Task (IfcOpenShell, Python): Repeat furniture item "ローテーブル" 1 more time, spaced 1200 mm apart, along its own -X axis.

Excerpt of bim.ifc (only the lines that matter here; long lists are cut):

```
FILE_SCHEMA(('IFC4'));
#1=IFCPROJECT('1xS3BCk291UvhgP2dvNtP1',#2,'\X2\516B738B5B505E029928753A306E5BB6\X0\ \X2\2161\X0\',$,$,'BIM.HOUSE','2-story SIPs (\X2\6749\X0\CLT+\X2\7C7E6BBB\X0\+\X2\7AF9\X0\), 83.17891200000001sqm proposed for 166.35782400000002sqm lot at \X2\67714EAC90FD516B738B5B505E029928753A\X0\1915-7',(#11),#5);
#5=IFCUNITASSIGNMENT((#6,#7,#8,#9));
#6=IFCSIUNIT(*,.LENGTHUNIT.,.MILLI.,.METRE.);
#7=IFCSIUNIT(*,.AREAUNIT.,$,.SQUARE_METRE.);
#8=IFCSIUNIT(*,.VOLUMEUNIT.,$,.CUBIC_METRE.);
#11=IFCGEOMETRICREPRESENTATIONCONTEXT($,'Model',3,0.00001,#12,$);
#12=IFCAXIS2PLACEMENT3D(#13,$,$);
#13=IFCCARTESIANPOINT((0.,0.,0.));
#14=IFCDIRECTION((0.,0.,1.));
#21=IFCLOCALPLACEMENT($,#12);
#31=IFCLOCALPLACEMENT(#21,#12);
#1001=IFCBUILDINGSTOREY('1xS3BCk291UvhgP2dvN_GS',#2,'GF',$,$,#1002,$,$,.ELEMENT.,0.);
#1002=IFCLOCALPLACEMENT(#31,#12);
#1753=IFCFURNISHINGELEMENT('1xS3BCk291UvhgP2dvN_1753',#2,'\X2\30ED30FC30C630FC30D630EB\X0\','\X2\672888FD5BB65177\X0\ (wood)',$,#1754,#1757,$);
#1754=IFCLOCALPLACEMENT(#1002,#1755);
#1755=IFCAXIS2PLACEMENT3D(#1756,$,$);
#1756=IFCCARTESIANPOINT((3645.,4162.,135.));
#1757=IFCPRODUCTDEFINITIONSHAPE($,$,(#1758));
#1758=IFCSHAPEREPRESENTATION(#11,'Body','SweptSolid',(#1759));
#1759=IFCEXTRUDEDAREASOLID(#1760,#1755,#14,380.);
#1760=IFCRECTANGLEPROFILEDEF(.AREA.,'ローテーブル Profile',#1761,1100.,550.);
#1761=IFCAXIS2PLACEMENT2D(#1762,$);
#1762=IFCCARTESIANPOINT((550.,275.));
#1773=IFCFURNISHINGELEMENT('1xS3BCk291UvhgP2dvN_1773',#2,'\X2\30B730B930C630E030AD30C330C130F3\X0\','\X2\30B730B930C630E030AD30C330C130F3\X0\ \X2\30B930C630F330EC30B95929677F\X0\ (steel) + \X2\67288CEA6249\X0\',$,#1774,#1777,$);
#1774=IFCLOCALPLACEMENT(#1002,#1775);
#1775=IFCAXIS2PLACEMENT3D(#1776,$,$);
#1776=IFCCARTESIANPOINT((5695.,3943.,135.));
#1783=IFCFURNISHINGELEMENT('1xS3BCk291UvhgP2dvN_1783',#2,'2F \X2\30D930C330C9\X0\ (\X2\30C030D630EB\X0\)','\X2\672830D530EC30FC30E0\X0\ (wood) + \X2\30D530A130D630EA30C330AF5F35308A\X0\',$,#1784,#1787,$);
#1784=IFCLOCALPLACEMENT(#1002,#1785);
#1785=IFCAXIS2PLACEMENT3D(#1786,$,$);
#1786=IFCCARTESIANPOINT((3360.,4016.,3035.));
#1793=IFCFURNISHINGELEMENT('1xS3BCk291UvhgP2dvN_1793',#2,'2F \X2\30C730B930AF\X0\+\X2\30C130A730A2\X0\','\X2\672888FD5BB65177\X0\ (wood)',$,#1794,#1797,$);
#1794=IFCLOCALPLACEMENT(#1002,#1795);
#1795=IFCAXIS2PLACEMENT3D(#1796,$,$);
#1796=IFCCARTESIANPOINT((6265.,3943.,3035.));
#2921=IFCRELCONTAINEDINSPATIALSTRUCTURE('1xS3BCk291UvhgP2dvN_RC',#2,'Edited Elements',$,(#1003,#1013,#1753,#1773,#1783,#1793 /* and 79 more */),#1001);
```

```python
import ifcopenshell
import ifcopenshell.api.geometry
import ifcopenshell.api.root
import ifcopenshell.util.element
import ifcopenshell.util.placement

model = ifcopenshell.open("bim.ifc")


def reuse_history(source, copy):
    """copy_class also copies each property set's owner history, people and application; keep the originals."""
    for rel in copy.IsDefinedBy:
        if rel.is_a("IfcRelDefinesByProperties") and (history := rel.RelatingPropertyDefinition.OwnerHistory):
            rel.RelatingPropertyDefinition.OwnerHistory = source.OwnerHistory
            ifcopenshell.util.element.remove_deep2(model, history)


source = model.by_guid("1xS3BCk291UvhgP2dvN_1753")
base = ifcopenshell.util.placement.get_local_placement(source.ObjectPlacement)
step = -base[:3, 0] * 1200.0

for i in range(1, 2):
    copy = ifcopenshell.api.root.copy_class(model, product=source)
    copy.Representation = ifcopenshell.util.element.copy_deep(
        model, source.Representation, exclude=["IfcGeometricRepresentationContext", "IfcRepresentationMap"]
    )
    reuse_history(source, copy)
    matrix = base.copy()
    matrix[:3, 3] += i * step
    print("added at", matrix[:3, 3].round(3) + 0.0)
    ifcopenshell.api.geometry.edit_object_placement(model, product=copy, matrix=matrix, is_si=False)

model.write("bim_updated.ifc")
```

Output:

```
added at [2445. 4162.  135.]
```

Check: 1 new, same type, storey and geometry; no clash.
